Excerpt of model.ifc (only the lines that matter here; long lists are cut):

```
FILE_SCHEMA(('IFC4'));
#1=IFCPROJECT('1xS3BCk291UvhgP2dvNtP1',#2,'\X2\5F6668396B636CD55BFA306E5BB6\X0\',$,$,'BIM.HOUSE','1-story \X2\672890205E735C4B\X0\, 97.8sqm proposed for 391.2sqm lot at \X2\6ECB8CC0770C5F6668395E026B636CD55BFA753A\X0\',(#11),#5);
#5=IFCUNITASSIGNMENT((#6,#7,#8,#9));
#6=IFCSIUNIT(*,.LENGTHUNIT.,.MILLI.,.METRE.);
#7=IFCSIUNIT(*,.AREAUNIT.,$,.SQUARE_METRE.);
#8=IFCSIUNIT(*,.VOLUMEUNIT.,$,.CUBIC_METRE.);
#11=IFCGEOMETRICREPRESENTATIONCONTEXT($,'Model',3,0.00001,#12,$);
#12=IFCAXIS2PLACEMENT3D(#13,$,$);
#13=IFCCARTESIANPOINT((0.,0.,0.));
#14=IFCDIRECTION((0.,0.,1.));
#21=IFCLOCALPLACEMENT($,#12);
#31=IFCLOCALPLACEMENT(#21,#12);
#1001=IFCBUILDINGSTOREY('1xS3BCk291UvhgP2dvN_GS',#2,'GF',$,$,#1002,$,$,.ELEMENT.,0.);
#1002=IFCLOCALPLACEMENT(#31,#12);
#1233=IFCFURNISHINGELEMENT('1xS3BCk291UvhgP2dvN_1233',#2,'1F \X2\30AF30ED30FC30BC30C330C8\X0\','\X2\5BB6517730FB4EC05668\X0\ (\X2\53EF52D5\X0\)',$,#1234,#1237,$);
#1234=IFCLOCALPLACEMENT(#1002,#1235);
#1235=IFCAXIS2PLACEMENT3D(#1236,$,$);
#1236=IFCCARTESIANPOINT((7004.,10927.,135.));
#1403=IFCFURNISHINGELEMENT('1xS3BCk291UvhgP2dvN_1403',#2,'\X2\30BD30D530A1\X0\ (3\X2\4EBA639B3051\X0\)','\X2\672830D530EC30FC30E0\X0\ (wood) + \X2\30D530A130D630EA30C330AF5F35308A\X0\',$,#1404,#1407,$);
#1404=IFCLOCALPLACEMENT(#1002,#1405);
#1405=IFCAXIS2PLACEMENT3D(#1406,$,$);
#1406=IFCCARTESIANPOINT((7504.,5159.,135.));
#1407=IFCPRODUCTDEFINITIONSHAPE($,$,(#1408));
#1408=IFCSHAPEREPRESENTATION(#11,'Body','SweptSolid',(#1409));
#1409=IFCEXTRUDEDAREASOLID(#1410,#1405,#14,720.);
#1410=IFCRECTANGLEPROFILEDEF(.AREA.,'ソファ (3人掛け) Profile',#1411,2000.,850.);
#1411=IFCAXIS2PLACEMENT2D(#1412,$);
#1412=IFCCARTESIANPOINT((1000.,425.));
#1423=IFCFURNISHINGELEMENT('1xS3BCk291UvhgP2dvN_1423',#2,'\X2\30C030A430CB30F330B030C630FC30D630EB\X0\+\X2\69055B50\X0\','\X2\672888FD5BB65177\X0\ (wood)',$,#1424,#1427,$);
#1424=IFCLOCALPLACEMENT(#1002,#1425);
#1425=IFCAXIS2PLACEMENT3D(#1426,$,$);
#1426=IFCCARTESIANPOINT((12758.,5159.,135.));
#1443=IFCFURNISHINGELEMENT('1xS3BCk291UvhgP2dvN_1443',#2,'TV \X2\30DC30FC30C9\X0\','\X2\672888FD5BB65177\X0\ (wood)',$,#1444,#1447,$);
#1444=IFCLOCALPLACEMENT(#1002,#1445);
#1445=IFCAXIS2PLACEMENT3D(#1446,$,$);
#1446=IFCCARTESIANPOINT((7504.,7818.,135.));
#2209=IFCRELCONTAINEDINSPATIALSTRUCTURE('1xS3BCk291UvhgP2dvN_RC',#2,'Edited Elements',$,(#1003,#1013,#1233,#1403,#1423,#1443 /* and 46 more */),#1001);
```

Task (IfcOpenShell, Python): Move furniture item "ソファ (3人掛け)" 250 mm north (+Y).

```python
import ifcopenshell
import ifcopenshell.api.geometry
import ifcopenshell.util.placement
import ifcopenshell.util.unit

model = ifcopenshell.open("model.ifc")
unit_scale = ifcopenshell.util.unit.calculate_unit_scale(model)

item = model.by_guid("1xS3BCk291UvhgP2dvN_1403")
matrix = ifcopenshell.util.placement.get_local_placement(item.ObjectPlacement)
matrix[1, 3] += 0.25 / unit_scale
ifcopenshell.api.geometry.edit_object_placement(model, product=item, matrix=matrix, is_si=False)

print(ifcopenshell.util.placement.get_local_placement(item.ObjectPlacement).round(3) + 0.0)

model.write("model_v2.ifc")
```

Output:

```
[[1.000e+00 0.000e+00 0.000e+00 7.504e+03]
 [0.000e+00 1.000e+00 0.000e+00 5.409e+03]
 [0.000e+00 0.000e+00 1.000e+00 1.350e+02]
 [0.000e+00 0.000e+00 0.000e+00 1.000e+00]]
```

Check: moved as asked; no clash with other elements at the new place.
